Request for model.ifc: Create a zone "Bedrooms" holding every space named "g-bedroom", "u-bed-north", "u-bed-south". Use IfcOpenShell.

First a look at what the model holds.

```python
import ifcopenshell

model = ifcopenshell.open("model.ifc")
print(model.schema)
seen = {}
for space in model.by_type("IfcSpace"):
    seen[space.LongName] = seen.get(space.LongName, 0) + 1
for name, count in sorted(seen.items(), key=str):
    print(count, "x", name)
print("zones:", [z.Name for z in model.by_type("IfcZone")][:20])
```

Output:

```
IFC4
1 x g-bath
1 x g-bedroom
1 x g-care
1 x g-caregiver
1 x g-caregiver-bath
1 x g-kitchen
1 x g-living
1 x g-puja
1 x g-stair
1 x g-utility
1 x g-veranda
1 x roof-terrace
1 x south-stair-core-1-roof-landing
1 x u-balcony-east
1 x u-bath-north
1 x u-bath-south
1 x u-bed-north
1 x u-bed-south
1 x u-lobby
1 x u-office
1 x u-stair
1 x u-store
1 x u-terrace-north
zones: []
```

```python
import ifcopenshell
import ifcopenshell.api.group
import ifcopenshell.api.root

model = ifcopenshell.open("model.ifc")

names = {"g-bedroom", "u-bed-north", "u-bed-south"}
spaces = [s for s in model.by_type("IfcSpace") if s.LongName in names]

zone = ifcopenshell.api.root.create_entity(model, ifc_class="IfcZone", name="Bedrooms")
ifcopenshell.api.group.assign_group(model, products=spaces, group=zone)
print(len(spaces), "spaces in", zone.Name)

model.write("model_updated.ifc")
```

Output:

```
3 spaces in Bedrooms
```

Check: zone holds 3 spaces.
